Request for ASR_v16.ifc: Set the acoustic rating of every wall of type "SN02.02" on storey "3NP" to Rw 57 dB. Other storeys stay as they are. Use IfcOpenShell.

First a look at what the model holds.

```python
import ifcopenshell
import ifcopenshell.util.element

model = ifcopenshell.open("ASR_v16.ifc")
print(model.schema)
storey = next(s for s in model.by_type("IfcBuildingStorey") if s.Name == "3NP")
walls = [e for e in ifcopenshell.util.element.get_decomposition(storey) if e.is_a("IfcWall")]
seen = {}
for e in walls:
    element_type = ifcopenshell.util.element.get_type(e)
    key = (element_type.Name if element_type != e and element_type else None, ifcopenshell.util.element.get_pset(e, "Pset_WallCommon", "AcousticRating"))
    seen[key] = seen.get(key, 0) + 1
for (name, value), count in sorted(seen.items(), key=str):
    print(count, "x", name, "|", value)
```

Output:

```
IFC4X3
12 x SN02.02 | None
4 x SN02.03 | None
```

```python
import ifcopenshell
import ifcopenshell.api.pset
import ifcopenshell.util.element

model = ifcopenshell.open("ASR_v16.ifc")

storey = next(s for s in model.by_type("IfcBuildingStorey") if s.Name == "3NP")
walls = [e for e in ifcopenshell.util.element.get_decomposition(storey) if e.is_a("IfcWall")]

count = 0
for e in walls:
    element_type = ifcopenshell.util.element.get_type(e)
    if element_type in (None, e) or element_type.Name != "SN02.02":
        continue
    # add_pset returns the element's existing set when there is one.
    pset = ifcopenshell.api.pset.add_pset(model, product=e, name="Pset_WallCommon")
    ifcopenshell.api.pset.edit_pset(model, pset=pset, properties={"AcousticRating": "Rw 57 dB"})
    count += 1

print(count, "walls updated")

model.write("ASR_v16_v2.ifc")
```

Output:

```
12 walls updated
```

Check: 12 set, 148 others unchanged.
